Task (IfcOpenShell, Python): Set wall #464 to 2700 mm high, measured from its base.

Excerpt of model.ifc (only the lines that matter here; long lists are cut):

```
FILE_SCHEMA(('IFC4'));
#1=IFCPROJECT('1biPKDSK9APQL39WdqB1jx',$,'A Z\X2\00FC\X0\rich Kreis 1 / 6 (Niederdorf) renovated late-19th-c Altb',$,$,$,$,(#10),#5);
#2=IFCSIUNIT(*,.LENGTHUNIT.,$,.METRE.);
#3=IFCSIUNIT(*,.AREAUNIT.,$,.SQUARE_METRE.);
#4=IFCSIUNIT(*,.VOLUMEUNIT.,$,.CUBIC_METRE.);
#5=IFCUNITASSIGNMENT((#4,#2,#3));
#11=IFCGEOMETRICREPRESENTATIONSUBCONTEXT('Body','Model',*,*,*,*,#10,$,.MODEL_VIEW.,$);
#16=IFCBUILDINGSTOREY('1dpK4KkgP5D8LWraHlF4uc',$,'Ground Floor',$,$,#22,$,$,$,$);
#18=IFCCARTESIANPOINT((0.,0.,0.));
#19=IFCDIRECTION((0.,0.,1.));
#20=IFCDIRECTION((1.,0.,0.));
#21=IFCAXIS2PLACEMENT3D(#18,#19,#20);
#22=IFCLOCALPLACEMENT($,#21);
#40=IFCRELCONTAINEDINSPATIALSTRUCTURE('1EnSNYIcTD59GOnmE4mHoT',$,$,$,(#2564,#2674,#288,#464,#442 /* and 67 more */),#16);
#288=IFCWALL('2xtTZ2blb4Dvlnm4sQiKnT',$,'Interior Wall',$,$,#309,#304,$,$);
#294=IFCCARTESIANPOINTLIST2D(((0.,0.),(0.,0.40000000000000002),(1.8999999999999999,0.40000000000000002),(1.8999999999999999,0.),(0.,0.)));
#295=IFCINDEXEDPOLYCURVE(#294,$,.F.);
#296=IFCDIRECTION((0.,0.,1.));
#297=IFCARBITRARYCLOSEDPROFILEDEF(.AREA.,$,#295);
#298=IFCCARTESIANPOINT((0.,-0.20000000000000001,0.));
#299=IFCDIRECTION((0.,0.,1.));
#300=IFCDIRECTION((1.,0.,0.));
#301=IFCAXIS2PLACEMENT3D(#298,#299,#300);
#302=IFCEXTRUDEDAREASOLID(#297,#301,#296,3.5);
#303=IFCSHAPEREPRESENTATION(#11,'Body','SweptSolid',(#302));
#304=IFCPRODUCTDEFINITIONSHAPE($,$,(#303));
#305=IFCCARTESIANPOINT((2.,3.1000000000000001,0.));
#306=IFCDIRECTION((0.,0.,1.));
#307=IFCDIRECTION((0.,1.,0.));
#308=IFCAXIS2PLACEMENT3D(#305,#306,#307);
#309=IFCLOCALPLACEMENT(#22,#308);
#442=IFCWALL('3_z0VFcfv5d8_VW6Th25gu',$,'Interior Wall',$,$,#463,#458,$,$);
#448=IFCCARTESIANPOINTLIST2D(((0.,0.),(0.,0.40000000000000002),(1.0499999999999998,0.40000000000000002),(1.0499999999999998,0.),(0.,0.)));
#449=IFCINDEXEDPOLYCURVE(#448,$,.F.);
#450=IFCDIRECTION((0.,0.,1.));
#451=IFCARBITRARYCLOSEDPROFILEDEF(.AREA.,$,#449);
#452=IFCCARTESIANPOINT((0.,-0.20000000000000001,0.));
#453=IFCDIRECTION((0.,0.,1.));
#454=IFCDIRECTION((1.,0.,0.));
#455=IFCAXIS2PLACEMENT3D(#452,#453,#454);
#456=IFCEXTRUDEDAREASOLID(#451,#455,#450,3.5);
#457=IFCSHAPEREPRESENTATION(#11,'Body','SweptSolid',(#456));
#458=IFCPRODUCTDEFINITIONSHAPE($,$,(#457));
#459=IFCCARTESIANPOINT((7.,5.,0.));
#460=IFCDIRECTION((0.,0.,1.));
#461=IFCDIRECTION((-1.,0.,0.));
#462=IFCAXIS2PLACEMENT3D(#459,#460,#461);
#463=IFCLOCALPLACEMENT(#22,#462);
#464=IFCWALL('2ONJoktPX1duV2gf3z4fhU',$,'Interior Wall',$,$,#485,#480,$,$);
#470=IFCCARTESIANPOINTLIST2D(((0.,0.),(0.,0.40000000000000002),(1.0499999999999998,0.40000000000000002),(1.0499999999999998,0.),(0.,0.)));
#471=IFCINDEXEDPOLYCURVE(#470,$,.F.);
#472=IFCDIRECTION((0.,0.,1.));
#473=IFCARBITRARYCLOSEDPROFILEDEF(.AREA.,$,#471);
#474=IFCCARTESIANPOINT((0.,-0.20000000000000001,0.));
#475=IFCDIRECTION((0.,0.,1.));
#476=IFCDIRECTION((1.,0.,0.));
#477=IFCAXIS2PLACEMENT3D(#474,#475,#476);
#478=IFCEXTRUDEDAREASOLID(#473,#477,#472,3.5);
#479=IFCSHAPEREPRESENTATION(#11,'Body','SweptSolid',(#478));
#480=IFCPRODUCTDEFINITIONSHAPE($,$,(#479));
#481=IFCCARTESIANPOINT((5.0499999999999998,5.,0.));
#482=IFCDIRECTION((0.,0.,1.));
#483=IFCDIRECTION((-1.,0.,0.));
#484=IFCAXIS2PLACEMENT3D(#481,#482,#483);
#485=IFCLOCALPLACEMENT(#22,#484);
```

```python
import ifcopenshell
import ifcopenshell.geom
import ifcopenshell.util.representation
import ifcopenshell.util.shape
import ifcopenshell.util.unit

model = ifcopenshell.open("model.ifc")
unit_scale = ifcopenshell.util.unit.calculate_unit_scale(model)
settings = ifcopenshell.geom.settings()


def volume(element):
    """Net volume in cubic metres, openings subtracted."""
    shape = ifcopenshell.geom.create_shape(settings, element)
    return ifcopenshell.util.shape.get_volume(shape.geometry)


wall = model.by_guid("2ONJoktPX1duV2gf3z4fhU")
before = volume(wall)

body = ifcopenshell.util.representation.get_representation(wall, "Model", "Body")
solid = body.Items[0]
old_height = solid.Depth
solid.Depth = 2.7 / unit_scale
after = volume(wall)

print(f"height {old_height:g} -> {solid.Depth:g}, volume {before:.3f} -> {after:.3f} m3")

model.write("model_v2.ifc")
```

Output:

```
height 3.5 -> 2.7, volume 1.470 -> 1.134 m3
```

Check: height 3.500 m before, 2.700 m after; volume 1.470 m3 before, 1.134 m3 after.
